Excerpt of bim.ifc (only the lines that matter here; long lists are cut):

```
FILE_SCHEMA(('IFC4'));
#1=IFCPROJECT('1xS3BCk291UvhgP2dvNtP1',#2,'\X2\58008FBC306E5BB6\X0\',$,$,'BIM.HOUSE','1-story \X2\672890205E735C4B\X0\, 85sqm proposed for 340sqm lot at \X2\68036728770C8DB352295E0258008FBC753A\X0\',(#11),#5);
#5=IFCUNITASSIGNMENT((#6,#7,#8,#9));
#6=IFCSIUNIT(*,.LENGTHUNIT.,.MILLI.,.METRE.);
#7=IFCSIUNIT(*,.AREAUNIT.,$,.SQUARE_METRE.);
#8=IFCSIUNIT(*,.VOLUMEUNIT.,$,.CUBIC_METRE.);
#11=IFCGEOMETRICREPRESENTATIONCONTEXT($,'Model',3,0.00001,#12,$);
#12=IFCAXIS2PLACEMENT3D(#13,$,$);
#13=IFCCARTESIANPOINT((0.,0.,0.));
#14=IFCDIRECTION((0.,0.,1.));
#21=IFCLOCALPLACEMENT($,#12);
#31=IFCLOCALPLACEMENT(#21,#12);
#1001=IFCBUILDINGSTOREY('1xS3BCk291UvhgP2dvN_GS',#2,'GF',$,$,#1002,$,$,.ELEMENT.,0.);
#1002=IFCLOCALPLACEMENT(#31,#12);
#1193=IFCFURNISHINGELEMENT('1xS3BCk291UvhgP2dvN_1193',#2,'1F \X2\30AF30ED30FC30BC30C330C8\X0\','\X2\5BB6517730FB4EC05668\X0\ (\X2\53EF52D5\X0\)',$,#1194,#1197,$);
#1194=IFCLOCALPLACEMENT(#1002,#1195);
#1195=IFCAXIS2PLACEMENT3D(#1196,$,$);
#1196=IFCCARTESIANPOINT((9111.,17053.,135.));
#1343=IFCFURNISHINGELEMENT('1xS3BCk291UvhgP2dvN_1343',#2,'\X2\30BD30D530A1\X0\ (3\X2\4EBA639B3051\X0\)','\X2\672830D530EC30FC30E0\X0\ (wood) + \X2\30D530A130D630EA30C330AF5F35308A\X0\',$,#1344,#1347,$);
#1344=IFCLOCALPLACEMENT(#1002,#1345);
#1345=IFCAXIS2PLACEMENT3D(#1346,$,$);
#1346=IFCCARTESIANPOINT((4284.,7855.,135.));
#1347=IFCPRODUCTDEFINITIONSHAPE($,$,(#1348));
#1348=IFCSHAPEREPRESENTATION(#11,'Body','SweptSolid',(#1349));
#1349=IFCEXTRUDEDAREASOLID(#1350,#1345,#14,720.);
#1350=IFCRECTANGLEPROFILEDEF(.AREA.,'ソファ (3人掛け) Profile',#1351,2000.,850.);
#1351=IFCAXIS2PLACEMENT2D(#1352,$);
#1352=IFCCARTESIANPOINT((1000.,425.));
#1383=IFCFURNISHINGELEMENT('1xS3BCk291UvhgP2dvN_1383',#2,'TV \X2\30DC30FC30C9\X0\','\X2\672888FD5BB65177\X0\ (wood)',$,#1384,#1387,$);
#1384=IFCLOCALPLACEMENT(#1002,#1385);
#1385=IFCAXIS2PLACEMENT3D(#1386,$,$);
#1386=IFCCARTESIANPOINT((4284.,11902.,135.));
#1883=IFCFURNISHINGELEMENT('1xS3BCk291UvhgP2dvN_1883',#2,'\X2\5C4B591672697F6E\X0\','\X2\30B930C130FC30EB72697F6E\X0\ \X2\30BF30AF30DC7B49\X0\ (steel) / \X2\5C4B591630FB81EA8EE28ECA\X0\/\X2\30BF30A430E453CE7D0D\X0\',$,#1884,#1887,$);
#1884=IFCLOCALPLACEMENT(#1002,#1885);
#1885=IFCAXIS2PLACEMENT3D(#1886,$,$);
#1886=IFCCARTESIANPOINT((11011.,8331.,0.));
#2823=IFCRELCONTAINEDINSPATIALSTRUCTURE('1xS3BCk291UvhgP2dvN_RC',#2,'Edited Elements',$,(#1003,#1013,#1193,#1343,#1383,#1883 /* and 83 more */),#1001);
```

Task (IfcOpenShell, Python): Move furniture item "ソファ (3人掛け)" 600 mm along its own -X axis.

```python
import ifcopenshell
import ifcopenshell.api.geometry
import ifcopenshell.util.placement
import ifcopenshell.util.unit

model = ifcopenshell.open("bim.ifc")
unit_scale = ifcopenshell.util.unit.calculate_unit_scale(model)

item = model.by_id(1343)
matrix = ifcopenshell.util.placement.get_local_placement(item.ObjectPlacement)
matrix[:3, 3] -= matrix[:3, 0] * 0.6 / unit_scale
ifcopenshell.api.geometry.edit_object_placement(model, product=item, matrix=matrix, is_si=False)

print(ifcopenshell.util.placement.get_local_placement(item.ObjectPlacement).round(3) + 0.0)

model.write("bim_rev.ifc")
```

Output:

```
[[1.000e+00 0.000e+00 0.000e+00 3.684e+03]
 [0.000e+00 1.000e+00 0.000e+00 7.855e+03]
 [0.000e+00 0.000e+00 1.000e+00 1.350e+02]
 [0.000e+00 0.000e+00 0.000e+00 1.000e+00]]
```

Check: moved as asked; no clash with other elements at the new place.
